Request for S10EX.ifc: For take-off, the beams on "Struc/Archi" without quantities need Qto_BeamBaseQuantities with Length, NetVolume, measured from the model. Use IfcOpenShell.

First a look at what the model holds.

```python
import ifcopenshell
import ifcopenshell.util.element
import ifcopenshell.util.unit

model = ifcopenshell.open("S10EX.ifc")
print(model.schema)
for unit_type in ("LENGTHUNIT", "AREAUNIT", "VOLUMEUNIT"):
    print(unit_type, ifcopenshell.util.unit.calculate_unit_scale(model, unit_type))
storey = next(s for s in model.by_type("IfcBuildingStorey") if s.Name == "Struc/Archi")
beams = [e for e in ifcopenshell.util.element.get_decomposition(storey) if e.is_a("IfcBeam")]
for e in sorted(beams, key=lambda e: e.id()):
    print(e.id(), e.is_a(), e.Name, list(ifcopenshell.util.element.get_psets(e, qtos_only=True)), sep=" | ")
```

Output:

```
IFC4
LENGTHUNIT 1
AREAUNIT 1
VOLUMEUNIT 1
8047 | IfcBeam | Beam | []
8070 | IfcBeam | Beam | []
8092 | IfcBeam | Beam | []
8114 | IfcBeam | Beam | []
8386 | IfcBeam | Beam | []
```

```python
import ifcopenshell
import ifcopenshell.api.pset
import ifcopenshell.geom
import ifcopenshell.util.element
import ifcopenshell.util.shape
import ifcopenshell.util.unit

model = ifcopenshell.open("S10EX.ifc")
unit_scale = ifcopenshell.util.unit.calculate_unit_scale(model)
volume_scale = ifcopenshell.util.unit.calculate_unit_scale(model, "VOLUMEUNIT")
settings = ifcopenshell.geom.settings()

storey = next(s for s in model.by_type("IfcBuildingStorey") if s.Name == "Struc/Archi")
beams = [e for e in ifcopenshell.util.element.get_decomposition(storey) if e.is_a("IfcBeam")]

for e in sorted(beams, key=lambda e: e.id()):
    if ifcopenshell.util.element.get_psets(e, qtos_only=True, should_inherit=False):
        continue
    # Geometry comes back in metres, in the element's own axes.
    shape = ifcopenshell.geom.create_shape(settings, e)
    values = {
        "Length": ifcopenshell.util.shape.get_max_xyz(shape.geometry) / unit_scale,
        "NetVolume": ifcopenshell.util.shape.get_volume(shape.geometry) / volume_scale,
    }
    qto = ifcopenshell.api.pset.add_qto(model, product=e, name="Qto_BeamBaseQuantities")
    ifcopenshell.api.pset.edit_qto(model, qto=qto, properties=values)
    print(e.id(), {k: round(v, 3) for k, v in values.items()})

model.write("S10EX_v2.ifc")
```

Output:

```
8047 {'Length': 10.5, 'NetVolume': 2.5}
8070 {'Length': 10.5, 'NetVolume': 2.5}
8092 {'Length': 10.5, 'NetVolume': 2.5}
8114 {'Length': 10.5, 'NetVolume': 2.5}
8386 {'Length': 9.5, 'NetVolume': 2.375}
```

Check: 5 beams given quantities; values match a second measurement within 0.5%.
